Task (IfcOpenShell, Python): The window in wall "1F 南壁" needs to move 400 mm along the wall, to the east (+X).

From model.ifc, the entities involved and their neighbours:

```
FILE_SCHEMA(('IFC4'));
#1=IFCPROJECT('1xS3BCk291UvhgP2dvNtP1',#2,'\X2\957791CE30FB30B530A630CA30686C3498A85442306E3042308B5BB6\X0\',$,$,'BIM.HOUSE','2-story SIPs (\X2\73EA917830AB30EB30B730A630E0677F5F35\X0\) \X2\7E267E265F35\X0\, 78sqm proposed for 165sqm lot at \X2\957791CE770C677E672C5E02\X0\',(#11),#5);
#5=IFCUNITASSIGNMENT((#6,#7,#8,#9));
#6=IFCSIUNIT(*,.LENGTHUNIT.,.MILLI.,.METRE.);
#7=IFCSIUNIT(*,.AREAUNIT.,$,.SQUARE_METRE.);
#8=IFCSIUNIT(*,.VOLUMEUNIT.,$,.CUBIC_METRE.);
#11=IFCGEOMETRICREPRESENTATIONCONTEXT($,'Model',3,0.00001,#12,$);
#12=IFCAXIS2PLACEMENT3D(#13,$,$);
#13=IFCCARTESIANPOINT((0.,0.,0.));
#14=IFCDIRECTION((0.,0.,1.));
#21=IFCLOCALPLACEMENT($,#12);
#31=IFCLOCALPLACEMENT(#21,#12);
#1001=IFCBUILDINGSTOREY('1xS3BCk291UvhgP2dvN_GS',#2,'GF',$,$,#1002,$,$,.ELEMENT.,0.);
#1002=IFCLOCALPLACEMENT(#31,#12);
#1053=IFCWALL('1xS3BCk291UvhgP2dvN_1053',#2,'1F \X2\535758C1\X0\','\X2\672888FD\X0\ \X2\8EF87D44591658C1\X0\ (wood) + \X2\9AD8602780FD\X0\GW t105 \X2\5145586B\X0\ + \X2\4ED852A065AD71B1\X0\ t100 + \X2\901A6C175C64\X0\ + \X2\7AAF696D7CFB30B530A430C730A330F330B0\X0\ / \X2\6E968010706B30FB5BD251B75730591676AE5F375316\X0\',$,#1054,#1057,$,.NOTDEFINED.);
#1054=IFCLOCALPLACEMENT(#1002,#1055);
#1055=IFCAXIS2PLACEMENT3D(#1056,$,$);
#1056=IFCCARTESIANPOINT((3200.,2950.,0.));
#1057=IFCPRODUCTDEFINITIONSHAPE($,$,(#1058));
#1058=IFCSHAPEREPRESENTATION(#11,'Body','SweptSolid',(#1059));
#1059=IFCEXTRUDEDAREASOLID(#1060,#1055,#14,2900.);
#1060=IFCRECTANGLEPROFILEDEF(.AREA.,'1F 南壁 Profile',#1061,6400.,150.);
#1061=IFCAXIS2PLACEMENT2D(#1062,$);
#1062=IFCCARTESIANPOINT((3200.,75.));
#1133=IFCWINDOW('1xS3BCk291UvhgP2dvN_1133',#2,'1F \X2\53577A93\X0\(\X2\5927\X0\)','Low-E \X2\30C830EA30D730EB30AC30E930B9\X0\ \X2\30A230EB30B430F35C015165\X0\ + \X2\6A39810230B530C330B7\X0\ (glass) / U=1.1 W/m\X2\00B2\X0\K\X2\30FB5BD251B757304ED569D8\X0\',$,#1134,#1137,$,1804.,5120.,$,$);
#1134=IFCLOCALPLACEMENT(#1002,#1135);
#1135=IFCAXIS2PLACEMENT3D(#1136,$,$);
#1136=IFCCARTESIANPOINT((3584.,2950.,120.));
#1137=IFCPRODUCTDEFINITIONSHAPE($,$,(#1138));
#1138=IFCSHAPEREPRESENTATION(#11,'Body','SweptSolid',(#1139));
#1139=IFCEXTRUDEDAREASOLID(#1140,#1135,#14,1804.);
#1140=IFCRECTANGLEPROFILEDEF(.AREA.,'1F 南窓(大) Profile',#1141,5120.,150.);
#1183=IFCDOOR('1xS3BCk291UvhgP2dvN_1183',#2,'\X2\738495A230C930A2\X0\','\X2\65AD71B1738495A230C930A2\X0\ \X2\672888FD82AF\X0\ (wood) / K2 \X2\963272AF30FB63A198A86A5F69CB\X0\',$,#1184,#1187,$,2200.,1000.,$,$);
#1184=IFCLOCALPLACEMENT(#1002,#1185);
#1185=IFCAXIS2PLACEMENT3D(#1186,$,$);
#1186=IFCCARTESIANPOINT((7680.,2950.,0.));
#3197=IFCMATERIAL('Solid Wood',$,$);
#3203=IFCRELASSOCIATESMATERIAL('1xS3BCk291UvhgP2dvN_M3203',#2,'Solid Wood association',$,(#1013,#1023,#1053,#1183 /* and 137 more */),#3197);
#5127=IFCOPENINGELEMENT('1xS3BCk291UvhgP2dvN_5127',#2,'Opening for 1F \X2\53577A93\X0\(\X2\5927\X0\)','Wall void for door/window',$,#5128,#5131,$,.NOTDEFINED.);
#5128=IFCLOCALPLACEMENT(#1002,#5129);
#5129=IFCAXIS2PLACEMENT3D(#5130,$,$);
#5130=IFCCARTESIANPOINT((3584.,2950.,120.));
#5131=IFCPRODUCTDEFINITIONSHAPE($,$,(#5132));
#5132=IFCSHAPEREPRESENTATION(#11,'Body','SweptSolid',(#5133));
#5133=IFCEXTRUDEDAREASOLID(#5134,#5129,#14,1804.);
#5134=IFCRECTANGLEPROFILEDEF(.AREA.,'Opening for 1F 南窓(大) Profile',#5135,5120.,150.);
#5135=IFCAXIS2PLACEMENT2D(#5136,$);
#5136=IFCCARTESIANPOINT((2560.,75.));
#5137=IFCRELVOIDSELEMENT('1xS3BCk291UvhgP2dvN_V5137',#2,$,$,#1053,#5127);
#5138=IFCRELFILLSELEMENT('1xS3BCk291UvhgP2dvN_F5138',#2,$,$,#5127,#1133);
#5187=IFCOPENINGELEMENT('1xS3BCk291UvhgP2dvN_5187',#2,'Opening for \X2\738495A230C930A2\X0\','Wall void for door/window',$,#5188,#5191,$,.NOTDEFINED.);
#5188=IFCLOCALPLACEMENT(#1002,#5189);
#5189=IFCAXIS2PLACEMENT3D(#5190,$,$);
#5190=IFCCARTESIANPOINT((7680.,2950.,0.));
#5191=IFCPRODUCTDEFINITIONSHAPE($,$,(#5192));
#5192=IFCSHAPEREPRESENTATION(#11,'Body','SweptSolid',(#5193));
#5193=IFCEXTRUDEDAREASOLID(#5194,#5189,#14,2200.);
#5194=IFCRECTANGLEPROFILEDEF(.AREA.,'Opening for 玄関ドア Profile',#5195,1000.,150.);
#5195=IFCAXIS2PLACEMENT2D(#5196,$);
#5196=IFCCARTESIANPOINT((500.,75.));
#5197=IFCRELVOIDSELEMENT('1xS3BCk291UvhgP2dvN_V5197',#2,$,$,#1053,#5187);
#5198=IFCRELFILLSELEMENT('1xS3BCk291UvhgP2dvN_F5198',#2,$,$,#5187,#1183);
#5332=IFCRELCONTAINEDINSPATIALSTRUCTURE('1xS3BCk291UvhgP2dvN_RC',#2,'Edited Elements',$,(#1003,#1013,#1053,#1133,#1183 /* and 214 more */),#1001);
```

```python
import ifcopenshell
import ifcopenshell.api.geometry
import ifcopenshell.util.placement

model = ifcopenshell.open("model.ifc")

window = model.by_guid("1xS3BCk291UvhgP2dvN_1133")
opening = window.FillsVoids[0].RelatingOpeningElement
wall = opening.VoidsElements[0].RelatingBuildingElement

wall_matrix = ifcopenshell.util.placement.get_local_placement(wall.ObjectPlacement)
shift = wall_matrix[:3, 0] * 400.0
before = ifcopenshell.util.placement.get_local_placement(window.ObjectPlacement)[:3, 3].copy()

# The window is not placed relative to its opening, so move both.
for product in (opening, window):
    matrix = ifcopenshell.util.placement.get_local_placement(product.ObjectPlacement)
    matrix[:3, 3] += shift
    ifcopenshell.api.geometry.edit_object_placement(model, product=product, matrix=matrix, is_si=False)

after = ifcopenshell.util.placement.get_local_placement(window.ObjectPlacement)[:3, 3]
print("window moved by", (after - before).round(3) + 0.0)

model.write("model_edited.ifc")
```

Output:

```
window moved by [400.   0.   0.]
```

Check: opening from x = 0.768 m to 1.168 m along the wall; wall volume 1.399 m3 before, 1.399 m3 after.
